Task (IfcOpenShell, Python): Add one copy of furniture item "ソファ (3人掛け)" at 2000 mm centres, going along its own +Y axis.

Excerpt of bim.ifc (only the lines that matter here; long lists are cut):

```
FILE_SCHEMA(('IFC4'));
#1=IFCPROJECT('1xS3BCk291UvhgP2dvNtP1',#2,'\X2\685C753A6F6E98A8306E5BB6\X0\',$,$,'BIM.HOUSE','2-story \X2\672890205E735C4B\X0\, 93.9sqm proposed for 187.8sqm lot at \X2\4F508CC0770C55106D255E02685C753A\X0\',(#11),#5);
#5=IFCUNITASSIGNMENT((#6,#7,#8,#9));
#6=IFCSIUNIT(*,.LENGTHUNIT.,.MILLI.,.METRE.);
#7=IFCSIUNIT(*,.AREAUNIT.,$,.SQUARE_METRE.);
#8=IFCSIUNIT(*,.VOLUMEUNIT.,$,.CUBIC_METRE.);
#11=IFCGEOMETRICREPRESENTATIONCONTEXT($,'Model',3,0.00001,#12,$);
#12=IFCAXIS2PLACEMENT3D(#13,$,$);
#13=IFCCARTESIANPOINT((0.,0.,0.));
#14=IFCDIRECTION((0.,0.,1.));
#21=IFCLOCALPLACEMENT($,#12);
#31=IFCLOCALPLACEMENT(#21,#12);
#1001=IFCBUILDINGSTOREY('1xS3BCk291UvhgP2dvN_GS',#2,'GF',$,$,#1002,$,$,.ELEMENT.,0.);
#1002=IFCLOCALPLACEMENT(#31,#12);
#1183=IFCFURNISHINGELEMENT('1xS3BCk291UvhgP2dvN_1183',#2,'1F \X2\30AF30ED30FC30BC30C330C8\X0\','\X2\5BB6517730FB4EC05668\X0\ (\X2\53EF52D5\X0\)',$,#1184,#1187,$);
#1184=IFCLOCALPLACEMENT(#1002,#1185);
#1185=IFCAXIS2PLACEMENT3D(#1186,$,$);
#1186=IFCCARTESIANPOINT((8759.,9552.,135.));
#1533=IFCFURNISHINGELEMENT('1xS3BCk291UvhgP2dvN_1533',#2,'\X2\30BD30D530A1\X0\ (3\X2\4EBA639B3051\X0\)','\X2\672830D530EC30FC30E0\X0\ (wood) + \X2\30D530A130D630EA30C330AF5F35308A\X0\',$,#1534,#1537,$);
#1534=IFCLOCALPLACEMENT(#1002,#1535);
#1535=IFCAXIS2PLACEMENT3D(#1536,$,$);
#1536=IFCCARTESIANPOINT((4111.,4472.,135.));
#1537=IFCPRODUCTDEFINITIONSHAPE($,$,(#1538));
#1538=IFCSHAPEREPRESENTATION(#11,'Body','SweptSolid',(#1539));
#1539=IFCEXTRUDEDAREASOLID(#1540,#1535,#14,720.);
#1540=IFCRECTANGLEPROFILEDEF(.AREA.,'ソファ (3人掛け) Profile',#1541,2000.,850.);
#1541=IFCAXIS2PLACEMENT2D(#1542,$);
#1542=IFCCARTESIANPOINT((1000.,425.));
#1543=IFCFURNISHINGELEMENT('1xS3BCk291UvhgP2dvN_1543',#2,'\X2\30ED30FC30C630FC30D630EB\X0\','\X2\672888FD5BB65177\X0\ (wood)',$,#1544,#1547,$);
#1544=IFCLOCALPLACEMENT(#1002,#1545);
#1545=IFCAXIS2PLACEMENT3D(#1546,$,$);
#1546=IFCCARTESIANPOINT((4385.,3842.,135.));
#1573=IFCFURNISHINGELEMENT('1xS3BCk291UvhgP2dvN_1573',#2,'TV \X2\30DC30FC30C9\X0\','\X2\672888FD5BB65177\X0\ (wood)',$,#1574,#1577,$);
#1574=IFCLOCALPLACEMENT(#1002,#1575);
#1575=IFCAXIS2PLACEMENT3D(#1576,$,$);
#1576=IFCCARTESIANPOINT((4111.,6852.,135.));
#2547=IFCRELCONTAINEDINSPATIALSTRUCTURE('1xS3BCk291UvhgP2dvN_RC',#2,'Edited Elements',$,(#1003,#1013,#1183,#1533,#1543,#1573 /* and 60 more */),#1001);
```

```python
import ifcopenshell
import ifcopenshell.api.geometry
import ifcopenshell.api.root
import ifcopenshell.util.element
import ifcopenshell.util.placement

model = ifcopenshell.open("bim.ifc")


def reuse_history(source, copy):
    """copy_class also copies each property set's owner history, people and application; keep the originals."""
    for rel in copy.IsDefinedBy:
        if rel.is_a("IfcRelDefinesByProperties") and (history := rel.RelatingPropertyDefinition.OwnerHistory):
            rel.RelatingPropertyDefinition.OwnerHistory = source.OwnerHistory
            ifcopenshell.util.element.remove_deep2(model, history)


source = model.by_id(1533)
base = ifcopenshell.util.placement.get_local_placement(source.ObjectPlacement)
step = base[:3, 1] * 2000.0

for i in range(1, 2):
    copy = ifcopenshell.api.root.copy_class(model, product=source)
    copy.Representation = ifcopenshell.util.element.copy_deep(
        model, source.Representation, exclude=["IfcGeometricRepresentationContext", "IfcRepresentationMap"]
    )
    reuse_history(source, copy)
    matrix = base.copy()
    matrix[:3, 3] += i * step
    print("added at", matrix[:3, 3].round(3) + 0.0)
    ifcopenshell.api.geometry.edit_object_placement(model, product=copy, matrix=matrix, is_si=False)

model.write("bim_rev.ifc")
```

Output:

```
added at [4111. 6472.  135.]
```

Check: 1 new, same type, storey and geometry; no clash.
